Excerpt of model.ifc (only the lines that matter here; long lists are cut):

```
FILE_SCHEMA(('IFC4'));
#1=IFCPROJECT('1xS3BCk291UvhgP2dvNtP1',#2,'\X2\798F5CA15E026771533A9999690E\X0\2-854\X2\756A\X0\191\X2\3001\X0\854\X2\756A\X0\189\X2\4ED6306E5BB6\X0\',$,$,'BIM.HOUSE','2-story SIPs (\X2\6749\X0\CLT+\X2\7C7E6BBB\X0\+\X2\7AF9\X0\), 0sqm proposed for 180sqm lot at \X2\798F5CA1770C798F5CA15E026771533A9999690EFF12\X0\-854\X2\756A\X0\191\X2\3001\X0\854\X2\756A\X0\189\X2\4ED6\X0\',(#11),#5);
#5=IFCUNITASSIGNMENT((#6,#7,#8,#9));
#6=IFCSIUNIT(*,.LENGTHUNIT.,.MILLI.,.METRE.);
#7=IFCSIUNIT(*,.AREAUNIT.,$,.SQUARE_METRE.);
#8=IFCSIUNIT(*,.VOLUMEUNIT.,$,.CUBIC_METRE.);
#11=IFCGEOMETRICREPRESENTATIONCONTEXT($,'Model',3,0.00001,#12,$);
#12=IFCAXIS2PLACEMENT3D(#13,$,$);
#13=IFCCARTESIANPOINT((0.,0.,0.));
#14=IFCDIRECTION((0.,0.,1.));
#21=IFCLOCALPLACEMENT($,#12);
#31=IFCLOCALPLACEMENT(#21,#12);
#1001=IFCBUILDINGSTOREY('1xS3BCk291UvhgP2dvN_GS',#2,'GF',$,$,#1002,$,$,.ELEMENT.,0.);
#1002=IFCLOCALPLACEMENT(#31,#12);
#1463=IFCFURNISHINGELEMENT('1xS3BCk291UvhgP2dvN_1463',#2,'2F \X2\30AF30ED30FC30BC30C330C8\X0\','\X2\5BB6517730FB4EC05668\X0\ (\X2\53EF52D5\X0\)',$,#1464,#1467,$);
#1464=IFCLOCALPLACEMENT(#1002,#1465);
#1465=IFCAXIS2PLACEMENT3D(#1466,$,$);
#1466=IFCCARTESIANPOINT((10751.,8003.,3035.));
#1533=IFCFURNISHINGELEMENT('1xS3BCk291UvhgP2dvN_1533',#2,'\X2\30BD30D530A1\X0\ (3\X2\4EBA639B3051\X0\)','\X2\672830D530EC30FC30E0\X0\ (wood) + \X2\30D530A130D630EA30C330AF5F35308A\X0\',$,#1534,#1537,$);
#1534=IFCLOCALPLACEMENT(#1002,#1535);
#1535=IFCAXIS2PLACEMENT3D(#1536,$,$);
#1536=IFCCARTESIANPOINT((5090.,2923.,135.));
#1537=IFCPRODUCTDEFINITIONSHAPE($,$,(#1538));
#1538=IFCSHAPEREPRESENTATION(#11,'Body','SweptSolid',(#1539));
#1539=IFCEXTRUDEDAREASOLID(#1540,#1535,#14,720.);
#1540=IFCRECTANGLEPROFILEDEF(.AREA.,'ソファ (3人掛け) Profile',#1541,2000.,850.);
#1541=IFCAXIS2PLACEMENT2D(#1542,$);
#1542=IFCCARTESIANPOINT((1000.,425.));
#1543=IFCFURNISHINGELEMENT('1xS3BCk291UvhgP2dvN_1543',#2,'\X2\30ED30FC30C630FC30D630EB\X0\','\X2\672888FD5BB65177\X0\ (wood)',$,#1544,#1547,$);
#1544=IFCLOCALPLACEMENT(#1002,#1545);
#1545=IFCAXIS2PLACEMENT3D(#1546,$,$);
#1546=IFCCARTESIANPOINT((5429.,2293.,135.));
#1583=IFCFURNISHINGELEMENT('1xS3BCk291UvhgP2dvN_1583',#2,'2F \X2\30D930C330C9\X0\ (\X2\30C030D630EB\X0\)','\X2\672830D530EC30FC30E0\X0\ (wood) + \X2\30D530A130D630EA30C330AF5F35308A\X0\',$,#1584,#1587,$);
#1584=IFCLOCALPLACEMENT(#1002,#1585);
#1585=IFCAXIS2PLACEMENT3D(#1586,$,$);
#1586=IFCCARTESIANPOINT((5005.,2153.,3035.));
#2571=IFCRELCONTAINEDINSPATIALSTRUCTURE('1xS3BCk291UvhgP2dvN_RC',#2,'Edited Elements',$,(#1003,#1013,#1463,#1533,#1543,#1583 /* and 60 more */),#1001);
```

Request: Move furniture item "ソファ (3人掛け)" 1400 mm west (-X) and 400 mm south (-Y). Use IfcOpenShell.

```python
import ifcopenshell
import ifcopenshell.api.geometry
import ifcopenshell.util.placement

model = ifcopenshell.open("model.ifc")

item = model.by_id(1533)
matrix = ifcopenshell.util.placement.get_local_placement(item.ObjectPlacement)
matrix[0, 3] -= 1400.0
matrix[1, 3] -= 400.0
ifcopenshell.api.geometry.edit_object_placement(model, product=item, matrix=matrix, is_si=False)

print(ifcopenshell.util.placement.get_local_placement(item.ObjectPlacement).round(3) + 0.0)

model.write("model_v2.ifc")
```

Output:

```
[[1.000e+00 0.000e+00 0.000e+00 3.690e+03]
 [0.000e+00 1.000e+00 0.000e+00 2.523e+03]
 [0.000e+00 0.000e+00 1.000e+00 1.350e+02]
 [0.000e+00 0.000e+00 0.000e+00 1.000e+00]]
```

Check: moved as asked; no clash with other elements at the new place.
